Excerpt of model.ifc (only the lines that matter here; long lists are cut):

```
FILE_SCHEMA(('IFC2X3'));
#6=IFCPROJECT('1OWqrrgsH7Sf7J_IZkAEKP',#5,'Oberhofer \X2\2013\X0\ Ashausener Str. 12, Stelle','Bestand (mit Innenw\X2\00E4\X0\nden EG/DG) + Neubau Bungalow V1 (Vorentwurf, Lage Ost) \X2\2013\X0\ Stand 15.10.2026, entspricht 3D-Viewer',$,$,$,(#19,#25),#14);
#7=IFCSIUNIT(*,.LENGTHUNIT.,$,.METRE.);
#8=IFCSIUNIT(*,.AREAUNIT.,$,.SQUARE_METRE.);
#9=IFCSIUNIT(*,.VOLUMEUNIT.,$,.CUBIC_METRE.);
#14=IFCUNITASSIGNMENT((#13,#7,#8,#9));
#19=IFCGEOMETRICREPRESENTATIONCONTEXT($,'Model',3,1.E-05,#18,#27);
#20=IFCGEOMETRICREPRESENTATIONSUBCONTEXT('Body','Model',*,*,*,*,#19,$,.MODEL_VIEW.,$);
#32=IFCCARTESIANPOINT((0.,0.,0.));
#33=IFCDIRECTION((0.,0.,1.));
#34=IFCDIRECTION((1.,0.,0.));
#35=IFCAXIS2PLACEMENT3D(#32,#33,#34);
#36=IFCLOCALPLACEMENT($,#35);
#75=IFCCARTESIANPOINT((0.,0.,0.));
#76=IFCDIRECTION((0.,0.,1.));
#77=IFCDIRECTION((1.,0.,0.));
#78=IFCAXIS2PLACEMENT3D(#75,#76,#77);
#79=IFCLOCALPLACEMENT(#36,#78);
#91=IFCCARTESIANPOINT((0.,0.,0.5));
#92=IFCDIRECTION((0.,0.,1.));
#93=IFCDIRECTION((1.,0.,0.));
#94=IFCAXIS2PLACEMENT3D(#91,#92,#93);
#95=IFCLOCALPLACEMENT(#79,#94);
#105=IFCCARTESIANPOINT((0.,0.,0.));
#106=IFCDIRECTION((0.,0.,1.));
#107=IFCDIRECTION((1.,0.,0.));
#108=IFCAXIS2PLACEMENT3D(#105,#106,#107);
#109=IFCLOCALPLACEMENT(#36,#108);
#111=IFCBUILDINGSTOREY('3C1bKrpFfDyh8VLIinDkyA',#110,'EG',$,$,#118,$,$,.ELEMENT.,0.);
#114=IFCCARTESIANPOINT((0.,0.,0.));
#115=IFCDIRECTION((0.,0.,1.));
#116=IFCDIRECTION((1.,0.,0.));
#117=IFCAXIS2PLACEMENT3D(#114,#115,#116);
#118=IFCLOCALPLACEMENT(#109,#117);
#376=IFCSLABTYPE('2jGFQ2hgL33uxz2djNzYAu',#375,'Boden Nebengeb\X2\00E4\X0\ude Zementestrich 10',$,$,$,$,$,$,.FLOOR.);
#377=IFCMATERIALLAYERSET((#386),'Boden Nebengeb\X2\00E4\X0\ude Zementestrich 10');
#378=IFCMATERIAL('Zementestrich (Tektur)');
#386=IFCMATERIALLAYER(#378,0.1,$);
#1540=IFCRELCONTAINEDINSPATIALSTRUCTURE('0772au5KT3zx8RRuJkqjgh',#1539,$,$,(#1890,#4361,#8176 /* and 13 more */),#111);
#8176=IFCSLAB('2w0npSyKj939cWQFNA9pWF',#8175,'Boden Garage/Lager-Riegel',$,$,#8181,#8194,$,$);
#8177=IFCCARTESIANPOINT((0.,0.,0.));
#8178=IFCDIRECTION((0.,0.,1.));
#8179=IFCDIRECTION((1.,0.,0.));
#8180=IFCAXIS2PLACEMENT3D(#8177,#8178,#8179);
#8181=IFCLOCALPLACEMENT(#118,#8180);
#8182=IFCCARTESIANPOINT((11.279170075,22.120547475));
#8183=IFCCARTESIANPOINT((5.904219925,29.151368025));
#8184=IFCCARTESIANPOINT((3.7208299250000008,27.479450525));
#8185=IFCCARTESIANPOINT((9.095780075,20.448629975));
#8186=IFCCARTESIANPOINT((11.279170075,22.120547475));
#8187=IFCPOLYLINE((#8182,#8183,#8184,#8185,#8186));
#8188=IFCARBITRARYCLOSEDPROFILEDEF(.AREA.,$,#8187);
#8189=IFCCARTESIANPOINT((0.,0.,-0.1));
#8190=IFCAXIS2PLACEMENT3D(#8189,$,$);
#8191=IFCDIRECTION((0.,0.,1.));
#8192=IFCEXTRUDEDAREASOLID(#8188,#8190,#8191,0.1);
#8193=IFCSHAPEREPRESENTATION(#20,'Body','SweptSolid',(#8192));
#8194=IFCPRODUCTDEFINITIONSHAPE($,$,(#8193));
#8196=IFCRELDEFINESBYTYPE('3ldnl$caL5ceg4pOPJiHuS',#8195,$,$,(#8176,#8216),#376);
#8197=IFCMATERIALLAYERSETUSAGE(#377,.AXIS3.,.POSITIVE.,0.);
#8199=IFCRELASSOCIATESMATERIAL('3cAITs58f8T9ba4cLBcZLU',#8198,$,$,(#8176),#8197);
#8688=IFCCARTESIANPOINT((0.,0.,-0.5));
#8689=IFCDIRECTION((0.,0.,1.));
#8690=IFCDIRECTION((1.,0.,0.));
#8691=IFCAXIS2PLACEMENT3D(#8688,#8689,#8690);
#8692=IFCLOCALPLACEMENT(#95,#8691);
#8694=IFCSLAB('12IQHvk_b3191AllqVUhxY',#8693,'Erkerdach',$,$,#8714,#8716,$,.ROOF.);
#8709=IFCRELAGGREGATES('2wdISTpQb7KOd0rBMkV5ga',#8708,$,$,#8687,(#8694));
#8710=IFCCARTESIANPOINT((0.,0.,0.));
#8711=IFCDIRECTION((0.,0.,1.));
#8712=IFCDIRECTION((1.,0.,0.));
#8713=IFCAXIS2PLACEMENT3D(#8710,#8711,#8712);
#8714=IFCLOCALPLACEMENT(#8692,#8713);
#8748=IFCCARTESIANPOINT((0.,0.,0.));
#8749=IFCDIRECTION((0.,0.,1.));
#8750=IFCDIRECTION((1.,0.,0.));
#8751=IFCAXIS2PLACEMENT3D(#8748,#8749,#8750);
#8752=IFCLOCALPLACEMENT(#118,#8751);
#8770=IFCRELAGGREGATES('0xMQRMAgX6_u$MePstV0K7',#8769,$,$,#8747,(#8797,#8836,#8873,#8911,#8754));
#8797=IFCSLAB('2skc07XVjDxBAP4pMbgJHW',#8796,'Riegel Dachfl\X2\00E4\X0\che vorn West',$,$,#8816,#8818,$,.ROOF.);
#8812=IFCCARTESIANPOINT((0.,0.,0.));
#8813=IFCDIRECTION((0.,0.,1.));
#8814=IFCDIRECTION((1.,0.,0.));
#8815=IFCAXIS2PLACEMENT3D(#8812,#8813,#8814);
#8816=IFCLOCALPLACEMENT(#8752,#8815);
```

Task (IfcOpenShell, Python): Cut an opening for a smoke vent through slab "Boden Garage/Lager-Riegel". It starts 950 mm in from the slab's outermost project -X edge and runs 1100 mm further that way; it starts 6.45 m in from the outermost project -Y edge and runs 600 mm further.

```python
import numpy as np
import ifcopenshell
import ifcopenshell.api.feature
import ifcopenshell.api.geometry
import ifcopenshell.api.root
import ifcopenshell.geom
import ifcopenshell.util.placement
import ifcopenshell.util.representation
import ifcopenshell.util.shape
import ifcopenshell.util.unit

model = ifcopenshell.open("model.ifc")
unit_scale = ifcopenshell.util.unit.calculate_unit_scale(model)
settings = ifcopenshell.geom.settings()


def volume(element):
    """Net volume in cubic metres, openings subtracted."""
    shape = ifcopenshell.geom.create_shape(settings, element)
    return ifcopenshell.util.shape.get_volume(shape.geometry)


slab = model.by_guid("2w0npSyKj939cWQFNA9pWF")
before = volume(slab)

# Extent in the slab's own axes, in metres. The edges named are its -X and -Y sides.
slab_shape = ifcopenshell.geom.create_shape(settings, slab)
vertices = ifcopenshell.util.shape.get_vertices(slab_shape.geometry)
x_min, y_min, bottom = vertices.min(axis=0)
top = vertices[:, 2].max()

opening = ifcopenshell.api.root.create_entity(model, ifc_class="IfcOpeningElement", name="Smoke vent opening")
context = ifcopenshell.util.representation.get_context(model, "Model", "Body", "MODEL_VIEW")
width, depth = 1.1, 0.6
outline = [(0.0, 0.0), (width, 0.0), (width, depth), (0.0, depth), (0.0, 0.0)]
# Overshoot both faces by 50 mm so the cut is clean.
shape = ifcopenshell.api.geometry.add_slab_representation(
    model, context=context, depth=top - bottom + 0.1, polyline=outline
)
ifcopenshell.api.geometry.assign_representation(model, product=opening, representation=shape)

matrix = ifcopenshell.util.placement.get_local_placement(slab.ObjectPlacement)
matrix[:, 3] = matrix @ np.append(np.array([x_min + 0.95, y_min + 6.45, bottom - 0.05]) / unit_scale, 1.0)
ifcopenshell.api.geometry.edit_object_placement(model, product=opening, matrix=matrix, is_si=False)
ifcopenshell.api.feature.add_feature(model, feature=opening, element=slab)

after = volume(slab)

print(f"slab volume {before:.3f} -> {after:.3f} m3")

model.write("model_rev.ifc")
```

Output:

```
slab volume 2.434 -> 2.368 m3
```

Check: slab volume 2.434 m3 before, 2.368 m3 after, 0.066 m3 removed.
